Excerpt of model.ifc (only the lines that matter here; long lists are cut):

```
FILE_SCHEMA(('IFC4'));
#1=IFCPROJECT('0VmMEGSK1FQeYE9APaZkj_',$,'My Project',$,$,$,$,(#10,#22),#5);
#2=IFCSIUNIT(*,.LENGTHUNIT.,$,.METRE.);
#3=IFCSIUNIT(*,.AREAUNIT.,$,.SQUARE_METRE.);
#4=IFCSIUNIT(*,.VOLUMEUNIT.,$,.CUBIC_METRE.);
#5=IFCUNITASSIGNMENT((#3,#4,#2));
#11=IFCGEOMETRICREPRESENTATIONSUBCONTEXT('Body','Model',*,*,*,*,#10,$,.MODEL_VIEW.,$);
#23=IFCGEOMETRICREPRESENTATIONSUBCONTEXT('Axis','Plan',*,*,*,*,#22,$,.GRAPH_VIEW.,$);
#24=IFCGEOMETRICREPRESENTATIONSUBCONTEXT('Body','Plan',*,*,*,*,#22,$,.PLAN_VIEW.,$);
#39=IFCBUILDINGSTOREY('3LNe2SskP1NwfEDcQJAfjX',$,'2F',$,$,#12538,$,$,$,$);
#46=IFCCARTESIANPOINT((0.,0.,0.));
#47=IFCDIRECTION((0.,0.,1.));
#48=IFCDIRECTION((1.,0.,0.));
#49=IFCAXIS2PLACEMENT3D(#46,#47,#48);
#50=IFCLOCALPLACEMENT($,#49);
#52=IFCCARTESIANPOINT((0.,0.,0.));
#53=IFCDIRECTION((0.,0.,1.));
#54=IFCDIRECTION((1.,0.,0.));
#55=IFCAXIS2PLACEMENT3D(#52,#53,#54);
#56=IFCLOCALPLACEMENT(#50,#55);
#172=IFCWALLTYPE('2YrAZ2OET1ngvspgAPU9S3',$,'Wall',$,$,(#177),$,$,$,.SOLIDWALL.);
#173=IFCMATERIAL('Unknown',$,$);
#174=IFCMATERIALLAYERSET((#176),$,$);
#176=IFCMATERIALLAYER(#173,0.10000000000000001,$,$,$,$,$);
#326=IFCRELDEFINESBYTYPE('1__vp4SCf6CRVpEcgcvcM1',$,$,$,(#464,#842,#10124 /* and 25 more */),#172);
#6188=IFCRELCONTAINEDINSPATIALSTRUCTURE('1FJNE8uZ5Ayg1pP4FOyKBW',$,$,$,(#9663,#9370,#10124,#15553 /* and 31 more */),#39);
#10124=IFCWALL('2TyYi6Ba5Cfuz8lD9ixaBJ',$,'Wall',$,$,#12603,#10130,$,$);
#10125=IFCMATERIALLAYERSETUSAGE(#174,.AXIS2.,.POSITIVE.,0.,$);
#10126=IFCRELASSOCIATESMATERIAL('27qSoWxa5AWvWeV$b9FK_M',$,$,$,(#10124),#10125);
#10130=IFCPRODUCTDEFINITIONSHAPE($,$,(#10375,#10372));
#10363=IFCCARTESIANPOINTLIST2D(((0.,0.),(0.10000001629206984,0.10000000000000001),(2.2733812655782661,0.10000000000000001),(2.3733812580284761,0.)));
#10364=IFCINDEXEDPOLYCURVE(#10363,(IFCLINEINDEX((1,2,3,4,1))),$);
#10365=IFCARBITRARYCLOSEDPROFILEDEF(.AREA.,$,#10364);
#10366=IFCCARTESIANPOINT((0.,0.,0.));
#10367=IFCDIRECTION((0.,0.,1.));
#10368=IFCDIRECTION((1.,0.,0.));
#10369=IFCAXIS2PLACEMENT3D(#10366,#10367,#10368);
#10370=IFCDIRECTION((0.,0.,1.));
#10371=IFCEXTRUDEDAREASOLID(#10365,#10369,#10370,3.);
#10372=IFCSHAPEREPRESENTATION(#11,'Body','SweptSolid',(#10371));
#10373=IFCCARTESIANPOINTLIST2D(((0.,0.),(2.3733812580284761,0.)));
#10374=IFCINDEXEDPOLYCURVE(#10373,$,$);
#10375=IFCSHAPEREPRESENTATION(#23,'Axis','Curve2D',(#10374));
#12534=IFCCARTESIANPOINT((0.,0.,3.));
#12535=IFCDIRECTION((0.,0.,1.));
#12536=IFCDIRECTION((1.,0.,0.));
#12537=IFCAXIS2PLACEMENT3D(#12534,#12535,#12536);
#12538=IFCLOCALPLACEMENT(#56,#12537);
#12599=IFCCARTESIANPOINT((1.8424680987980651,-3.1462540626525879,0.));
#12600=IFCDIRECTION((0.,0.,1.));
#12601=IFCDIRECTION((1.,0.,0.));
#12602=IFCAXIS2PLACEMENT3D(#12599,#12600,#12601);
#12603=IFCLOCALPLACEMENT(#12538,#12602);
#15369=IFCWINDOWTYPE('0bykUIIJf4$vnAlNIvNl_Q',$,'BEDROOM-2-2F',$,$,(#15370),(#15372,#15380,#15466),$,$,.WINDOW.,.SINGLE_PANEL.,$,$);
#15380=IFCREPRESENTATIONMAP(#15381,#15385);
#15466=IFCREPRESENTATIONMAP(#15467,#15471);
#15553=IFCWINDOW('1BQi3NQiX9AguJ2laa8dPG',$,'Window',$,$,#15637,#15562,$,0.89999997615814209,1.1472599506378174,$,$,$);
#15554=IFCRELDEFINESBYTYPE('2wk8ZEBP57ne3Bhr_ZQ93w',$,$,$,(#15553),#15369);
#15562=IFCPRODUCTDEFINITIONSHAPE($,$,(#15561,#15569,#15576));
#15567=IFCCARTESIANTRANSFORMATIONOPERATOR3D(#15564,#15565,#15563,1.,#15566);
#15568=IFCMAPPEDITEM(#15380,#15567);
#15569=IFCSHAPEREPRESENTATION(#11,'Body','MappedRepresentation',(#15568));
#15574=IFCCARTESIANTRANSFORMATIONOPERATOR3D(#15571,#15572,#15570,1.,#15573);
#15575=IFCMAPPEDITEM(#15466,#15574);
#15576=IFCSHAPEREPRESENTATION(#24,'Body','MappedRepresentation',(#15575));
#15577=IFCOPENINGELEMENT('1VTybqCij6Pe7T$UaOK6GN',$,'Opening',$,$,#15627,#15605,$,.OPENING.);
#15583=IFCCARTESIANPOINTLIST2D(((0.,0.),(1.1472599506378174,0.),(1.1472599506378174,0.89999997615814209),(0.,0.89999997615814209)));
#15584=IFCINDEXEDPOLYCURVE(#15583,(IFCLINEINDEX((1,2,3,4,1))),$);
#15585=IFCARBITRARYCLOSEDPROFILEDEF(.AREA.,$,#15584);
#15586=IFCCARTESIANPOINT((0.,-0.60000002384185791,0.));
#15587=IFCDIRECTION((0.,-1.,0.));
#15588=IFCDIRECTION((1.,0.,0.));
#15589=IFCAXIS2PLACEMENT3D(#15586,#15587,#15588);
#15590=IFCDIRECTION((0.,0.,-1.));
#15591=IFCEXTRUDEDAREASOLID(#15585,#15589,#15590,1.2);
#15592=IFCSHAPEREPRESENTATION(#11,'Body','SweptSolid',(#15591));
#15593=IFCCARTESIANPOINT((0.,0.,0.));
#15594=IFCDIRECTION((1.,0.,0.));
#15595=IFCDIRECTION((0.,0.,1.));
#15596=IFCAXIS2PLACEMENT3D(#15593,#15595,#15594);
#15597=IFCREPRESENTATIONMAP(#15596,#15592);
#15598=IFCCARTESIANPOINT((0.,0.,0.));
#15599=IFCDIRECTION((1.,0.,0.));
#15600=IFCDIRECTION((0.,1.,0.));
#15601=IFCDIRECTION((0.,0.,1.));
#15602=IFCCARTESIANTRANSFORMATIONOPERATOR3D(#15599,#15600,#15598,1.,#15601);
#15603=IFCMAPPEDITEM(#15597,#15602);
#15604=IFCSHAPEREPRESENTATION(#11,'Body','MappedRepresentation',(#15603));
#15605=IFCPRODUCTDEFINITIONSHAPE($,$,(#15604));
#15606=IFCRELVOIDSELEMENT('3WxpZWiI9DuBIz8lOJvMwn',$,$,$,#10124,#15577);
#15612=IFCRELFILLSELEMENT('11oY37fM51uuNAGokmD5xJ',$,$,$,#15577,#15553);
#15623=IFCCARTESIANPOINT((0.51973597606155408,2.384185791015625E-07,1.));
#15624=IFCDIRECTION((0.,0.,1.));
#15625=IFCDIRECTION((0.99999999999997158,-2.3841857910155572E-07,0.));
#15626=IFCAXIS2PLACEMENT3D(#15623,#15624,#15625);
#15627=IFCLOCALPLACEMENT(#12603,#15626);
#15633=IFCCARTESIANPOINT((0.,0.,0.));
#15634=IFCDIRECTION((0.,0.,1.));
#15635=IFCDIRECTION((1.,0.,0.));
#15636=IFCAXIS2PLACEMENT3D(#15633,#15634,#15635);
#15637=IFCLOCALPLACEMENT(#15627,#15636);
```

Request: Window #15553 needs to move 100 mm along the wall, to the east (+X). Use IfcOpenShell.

```python
import ifcopenshell
import ifcopenshell.api.geometry
import ifcopenshell.util.placement

model = ifcopenshell.open("model.ifc")

window = model.by_guid("1BQi3NQiX9AguJ2laa8dPG")
opening = window.FillsVoids[0].RelatingOpeningElement
wall = opening.VoidsElements[0].RelatingBuildingElement

wall_matrix = ifcopenshell.util.placement.get_local_placement(wall.ObjectPlacement)
shift = wall_matrix[:3, 0] * 0.1
before = ifcopenshell.util.placement.get_local_placement(window.ObjectPlacement)[:3, 3].copy()

# The window is placed relative to its opening, so it follows when the opening moves.
matrix = ifcopenshell.util.placement.get_local_placement(opening.ObjectPlacement)
matrix[:3, 3] += shift
ifcopenshell.api.geometry.edit_object_placement(
    model, product=opening, matrix=matrix, is_si=False, should_transform_children=True
)

after = ifcopenshell.util.placement.get_local_placement(window.ObjectPlacement)[:3, 3]
print("window moved by", (after - before).round(3) + 0.0)

model.write("model_edited.ifc")
```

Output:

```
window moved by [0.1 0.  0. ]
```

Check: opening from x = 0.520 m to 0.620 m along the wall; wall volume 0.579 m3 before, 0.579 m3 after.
